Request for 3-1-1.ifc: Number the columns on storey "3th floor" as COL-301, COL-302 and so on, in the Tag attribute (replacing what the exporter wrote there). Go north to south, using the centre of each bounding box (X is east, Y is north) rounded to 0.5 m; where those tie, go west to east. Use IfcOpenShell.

First a look at what the model holds.

```python
import ifcopenshell
import ifcopenshell.util.element
import ifcopenshell.util.placement

model = ifcopenshell.open("3-1-1.ifc")
print(model.schema)
storey = next(s for s in model.by_type("IfcBuildingStorey") if s.Name == "3th floor")
columns = [e for e in ifcopenshell.util.element.get_decomposition(storey) if e.is_a("IfcColumn")]
for e in sorted(columns, key=lambda e: e.id()):
    origin = ifcopenshell.util.placement.get_local_placement(e.ObjectPlacement)[:3, 3]
    print(e.id(), e.Tag, e.Name, origin.round(2) + 0.0, sep=" | ")
```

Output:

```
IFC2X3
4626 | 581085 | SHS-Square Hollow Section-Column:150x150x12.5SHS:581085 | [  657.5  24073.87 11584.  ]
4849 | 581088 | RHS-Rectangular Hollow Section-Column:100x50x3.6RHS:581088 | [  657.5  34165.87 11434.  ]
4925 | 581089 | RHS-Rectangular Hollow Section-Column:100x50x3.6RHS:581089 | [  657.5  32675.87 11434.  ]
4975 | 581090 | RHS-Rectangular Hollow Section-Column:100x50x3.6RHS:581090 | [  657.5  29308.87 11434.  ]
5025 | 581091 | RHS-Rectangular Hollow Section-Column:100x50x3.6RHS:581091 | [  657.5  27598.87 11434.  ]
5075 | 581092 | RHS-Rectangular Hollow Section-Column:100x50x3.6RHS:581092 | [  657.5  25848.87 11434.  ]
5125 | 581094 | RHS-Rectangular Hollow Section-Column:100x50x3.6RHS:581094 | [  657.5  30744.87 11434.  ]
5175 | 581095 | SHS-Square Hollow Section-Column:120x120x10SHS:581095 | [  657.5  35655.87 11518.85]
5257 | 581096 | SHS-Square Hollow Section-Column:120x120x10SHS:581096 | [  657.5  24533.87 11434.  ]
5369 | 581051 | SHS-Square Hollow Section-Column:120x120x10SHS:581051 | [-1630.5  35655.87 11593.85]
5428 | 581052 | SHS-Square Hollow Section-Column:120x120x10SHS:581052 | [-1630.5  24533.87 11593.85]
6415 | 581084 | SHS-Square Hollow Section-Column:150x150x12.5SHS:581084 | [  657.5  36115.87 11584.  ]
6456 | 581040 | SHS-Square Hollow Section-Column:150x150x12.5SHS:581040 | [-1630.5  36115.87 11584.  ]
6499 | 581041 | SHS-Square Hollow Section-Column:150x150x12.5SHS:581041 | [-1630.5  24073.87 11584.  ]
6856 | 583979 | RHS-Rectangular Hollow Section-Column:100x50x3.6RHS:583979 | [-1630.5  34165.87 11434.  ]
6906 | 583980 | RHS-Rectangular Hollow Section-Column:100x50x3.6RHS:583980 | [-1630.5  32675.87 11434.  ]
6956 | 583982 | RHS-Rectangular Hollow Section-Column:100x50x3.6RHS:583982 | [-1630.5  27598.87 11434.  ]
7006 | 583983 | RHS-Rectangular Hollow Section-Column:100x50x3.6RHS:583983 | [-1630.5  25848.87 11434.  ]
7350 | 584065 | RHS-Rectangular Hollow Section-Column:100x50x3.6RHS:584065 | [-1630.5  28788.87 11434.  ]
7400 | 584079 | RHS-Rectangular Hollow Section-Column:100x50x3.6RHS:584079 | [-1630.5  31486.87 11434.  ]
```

```python
import ifcopenshell
import ifcopenshell.geom
import ifcopenshell.util.element
import ifcopenshell.util.shape

model = ifcopenshell.open("3-1-1.ifc")
settings = ifcopenshell.geom.settings()
settings.set("use-world-coords", True)


def centre(element):
    shape = ifcopenshell.geom.create_shape(settings, element)
    return ifcopenshell.util.shape.get_bbox_centroid(shape.geometry)


storey = next(s for s in model.by_type("IfcBuildingStorey") if s.Name == "3th floor")
columns = [e for e in ifcopenshell.util.element.get_decomposition(storey) if e.is_a("IfcColumn")]

# Insertion points can sit at a corner or the storey origin, so sort by the geometry (in metres).
centres = {e: centre(e) for e in columns}
columns.sort(key=lambda e: (-round(centres[e][1] / 0.5), centres[e][0]))

for i, e in enumerate(columns, start=1):
    number = f"COL-3{i:02d}"
    e.Tag = number
    print(e.id(), number)

model.write("3-1-1-out.ifc")
```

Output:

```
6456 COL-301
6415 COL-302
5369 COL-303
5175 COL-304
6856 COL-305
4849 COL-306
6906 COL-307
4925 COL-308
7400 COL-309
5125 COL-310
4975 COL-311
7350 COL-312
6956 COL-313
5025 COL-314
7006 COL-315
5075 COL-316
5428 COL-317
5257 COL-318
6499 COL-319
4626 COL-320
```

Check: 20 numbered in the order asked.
